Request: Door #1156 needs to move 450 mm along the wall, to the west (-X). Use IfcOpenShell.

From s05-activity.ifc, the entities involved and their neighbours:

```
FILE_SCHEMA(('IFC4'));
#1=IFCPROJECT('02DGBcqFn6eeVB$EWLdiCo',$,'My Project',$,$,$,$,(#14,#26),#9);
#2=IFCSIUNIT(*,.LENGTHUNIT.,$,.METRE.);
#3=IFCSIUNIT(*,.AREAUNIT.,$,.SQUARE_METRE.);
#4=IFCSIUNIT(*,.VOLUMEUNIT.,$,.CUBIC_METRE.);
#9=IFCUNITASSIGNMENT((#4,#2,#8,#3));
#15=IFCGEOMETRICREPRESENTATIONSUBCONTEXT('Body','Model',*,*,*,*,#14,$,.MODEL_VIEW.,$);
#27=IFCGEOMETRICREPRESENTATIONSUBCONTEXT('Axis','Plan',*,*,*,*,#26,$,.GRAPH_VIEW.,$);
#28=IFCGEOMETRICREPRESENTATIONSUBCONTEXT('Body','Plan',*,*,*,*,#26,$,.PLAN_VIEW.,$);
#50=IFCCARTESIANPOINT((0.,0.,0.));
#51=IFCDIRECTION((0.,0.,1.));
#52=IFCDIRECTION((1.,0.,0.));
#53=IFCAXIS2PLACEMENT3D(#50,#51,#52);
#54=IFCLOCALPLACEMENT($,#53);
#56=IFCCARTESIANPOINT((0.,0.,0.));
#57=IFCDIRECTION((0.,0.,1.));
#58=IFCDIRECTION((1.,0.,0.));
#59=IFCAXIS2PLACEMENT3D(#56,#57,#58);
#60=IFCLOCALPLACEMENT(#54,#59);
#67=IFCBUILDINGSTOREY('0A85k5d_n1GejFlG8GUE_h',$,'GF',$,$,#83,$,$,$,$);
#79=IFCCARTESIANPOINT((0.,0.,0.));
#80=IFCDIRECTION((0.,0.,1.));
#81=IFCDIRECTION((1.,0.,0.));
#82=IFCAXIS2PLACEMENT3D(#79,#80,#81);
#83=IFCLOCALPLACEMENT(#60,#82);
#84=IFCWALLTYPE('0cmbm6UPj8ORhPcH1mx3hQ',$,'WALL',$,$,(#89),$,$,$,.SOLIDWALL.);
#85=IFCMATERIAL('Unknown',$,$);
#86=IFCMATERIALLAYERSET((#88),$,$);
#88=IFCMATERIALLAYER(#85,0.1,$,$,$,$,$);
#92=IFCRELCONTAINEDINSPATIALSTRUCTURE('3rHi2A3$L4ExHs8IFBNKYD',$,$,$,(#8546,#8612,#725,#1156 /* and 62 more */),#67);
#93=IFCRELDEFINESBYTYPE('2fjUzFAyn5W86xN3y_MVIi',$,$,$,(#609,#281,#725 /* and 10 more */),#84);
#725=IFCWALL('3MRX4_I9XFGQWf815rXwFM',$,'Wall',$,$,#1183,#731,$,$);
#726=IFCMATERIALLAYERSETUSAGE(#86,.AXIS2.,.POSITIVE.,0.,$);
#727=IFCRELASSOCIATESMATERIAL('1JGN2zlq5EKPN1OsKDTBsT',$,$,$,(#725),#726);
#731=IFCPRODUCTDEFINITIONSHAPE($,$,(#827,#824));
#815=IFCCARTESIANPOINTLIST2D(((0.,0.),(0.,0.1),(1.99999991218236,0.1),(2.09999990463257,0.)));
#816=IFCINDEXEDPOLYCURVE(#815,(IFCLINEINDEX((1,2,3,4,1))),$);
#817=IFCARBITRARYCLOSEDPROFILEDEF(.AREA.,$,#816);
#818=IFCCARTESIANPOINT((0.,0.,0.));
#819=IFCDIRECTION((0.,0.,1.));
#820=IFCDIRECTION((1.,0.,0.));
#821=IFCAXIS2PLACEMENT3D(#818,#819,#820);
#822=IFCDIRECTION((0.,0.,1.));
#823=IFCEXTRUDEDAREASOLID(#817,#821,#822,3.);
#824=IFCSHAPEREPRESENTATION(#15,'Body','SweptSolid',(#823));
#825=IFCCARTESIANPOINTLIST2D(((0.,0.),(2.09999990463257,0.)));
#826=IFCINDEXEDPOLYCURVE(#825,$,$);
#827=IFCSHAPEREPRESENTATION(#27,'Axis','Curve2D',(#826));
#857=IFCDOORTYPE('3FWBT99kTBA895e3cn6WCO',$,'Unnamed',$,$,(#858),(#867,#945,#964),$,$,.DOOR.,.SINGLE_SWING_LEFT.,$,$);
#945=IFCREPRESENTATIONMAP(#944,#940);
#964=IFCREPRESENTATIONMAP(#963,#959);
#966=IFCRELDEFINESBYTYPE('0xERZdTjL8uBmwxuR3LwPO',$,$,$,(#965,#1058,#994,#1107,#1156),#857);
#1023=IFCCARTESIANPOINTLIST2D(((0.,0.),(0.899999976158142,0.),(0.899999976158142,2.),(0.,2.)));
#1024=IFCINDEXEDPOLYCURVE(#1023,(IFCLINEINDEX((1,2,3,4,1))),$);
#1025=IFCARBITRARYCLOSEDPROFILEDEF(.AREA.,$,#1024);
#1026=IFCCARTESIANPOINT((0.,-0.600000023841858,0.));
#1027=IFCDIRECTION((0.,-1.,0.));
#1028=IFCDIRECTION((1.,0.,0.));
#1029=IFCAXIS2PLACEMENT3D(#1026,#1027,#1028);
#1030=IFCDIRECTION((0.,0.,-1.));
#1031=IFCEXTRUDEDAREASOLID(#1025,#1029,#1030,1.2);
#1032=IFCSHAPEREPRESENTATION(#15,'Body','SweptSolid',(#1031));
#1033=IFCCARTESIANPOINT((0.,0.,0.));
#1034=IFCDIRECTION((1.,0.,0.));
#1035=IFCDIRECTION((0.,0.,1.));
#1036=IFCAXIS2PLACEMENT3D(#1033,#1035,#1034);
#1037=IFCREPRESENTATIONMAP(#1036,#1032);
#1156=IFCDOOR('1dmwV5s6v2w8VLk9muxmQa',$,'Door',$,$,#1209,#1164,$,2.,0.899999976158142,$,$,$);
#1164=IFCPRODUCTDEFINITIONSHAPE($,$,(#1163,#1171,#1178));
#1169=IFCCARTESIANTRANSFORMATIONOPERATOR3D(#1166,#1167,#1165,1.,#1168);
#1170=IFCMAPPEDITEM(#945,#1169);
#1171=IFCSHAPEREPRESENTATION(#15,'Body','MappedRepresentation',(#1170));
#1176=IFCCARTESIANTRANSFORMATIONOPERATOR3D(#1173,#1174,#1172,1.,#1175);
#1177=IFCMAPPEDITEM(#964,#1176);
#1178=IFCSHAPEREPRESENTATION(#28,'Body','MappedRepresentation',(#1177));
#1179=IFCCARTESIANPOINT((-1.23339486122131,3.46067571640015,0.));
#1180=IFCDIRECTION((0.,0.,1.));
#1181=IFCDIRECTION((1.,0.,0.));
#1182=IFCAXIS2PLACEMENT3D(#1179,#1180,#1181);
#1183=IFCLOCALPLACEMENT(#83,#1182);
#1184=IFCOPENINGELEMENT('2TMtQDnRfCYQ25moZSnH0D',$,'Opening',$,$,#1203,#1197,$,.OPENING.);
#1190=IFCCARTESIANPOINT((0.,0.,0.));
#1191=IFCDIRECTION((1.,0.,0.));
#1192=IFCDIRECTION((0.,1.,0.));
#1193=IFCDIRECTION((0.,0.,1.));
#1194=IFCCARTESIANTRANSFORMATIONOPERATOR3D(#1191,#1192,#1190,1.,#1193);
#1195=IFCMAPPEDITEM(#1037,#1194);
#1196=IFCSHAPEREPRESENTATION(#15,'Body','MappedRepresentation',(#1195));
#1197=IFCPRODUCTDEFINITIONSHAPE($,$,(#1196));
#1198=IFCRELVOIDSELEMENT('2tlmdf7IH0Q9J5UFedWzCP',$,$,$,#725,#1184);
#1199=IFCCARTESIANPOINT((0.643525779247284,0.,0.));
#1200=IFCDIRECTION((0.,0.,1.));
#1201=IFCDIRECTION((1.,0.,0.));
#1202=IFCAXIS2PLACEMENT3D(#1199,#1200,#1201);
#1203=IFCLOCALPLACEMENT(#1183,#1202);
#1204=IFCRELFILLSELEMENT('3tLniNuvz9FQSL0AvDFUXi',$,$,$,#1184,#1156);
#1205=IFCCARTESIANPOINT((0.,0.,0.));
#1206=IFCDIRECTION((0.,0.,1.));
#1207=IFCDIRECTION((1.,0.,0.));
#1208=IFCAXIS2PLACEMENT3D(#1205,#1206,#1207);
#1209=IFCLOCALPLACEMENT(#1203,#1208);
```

```python
import ifcopenshell
import ifcopenshell.api.geometry
import ifcopenshell.util.placement

model = ifcopenshell.open("s05-activity.ifc")

door = model.by_guid("1dmwV5s6v2w8VLk9muxmQa")
opening = door.FillsVoids[0].RelatingOpeningElement
wall = opening.VoidsElements[0].RelatingBuildingElement

wall_matrix = ifcopenshell.util.placement.get_local_placement(wall.ObjectPlacement)
shift = wall_matrix[:3, 0] * -0.45
before = ifcopenshell.util.placement.get_local_placement(door.ObjectPlacement)[:3, 3].copy()

# The door is placed relative to its opening, so it follows when the opening moves.
matrix = ifcopenshell.util.placement.get_local_placement(opening.ObjectPlacement)
matrix[:3, 3] += shift
ifcopenshell.api.geometry.edit_object_placement(
    model, product=opening, matrix=matrix, is_si=False, should_transform_children=True
)

after = ifcopenshell.util.placement.get_local_placement(door.ObjectPlacement)[:3, 3]
print("door moved by", (after - before).round(3) + 0.0)

model.write("s05-activity_updated.ifc")
```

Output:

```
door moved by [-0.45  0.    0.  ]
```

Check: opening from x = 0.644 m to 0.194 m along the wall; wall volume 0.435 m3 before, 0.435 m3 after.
